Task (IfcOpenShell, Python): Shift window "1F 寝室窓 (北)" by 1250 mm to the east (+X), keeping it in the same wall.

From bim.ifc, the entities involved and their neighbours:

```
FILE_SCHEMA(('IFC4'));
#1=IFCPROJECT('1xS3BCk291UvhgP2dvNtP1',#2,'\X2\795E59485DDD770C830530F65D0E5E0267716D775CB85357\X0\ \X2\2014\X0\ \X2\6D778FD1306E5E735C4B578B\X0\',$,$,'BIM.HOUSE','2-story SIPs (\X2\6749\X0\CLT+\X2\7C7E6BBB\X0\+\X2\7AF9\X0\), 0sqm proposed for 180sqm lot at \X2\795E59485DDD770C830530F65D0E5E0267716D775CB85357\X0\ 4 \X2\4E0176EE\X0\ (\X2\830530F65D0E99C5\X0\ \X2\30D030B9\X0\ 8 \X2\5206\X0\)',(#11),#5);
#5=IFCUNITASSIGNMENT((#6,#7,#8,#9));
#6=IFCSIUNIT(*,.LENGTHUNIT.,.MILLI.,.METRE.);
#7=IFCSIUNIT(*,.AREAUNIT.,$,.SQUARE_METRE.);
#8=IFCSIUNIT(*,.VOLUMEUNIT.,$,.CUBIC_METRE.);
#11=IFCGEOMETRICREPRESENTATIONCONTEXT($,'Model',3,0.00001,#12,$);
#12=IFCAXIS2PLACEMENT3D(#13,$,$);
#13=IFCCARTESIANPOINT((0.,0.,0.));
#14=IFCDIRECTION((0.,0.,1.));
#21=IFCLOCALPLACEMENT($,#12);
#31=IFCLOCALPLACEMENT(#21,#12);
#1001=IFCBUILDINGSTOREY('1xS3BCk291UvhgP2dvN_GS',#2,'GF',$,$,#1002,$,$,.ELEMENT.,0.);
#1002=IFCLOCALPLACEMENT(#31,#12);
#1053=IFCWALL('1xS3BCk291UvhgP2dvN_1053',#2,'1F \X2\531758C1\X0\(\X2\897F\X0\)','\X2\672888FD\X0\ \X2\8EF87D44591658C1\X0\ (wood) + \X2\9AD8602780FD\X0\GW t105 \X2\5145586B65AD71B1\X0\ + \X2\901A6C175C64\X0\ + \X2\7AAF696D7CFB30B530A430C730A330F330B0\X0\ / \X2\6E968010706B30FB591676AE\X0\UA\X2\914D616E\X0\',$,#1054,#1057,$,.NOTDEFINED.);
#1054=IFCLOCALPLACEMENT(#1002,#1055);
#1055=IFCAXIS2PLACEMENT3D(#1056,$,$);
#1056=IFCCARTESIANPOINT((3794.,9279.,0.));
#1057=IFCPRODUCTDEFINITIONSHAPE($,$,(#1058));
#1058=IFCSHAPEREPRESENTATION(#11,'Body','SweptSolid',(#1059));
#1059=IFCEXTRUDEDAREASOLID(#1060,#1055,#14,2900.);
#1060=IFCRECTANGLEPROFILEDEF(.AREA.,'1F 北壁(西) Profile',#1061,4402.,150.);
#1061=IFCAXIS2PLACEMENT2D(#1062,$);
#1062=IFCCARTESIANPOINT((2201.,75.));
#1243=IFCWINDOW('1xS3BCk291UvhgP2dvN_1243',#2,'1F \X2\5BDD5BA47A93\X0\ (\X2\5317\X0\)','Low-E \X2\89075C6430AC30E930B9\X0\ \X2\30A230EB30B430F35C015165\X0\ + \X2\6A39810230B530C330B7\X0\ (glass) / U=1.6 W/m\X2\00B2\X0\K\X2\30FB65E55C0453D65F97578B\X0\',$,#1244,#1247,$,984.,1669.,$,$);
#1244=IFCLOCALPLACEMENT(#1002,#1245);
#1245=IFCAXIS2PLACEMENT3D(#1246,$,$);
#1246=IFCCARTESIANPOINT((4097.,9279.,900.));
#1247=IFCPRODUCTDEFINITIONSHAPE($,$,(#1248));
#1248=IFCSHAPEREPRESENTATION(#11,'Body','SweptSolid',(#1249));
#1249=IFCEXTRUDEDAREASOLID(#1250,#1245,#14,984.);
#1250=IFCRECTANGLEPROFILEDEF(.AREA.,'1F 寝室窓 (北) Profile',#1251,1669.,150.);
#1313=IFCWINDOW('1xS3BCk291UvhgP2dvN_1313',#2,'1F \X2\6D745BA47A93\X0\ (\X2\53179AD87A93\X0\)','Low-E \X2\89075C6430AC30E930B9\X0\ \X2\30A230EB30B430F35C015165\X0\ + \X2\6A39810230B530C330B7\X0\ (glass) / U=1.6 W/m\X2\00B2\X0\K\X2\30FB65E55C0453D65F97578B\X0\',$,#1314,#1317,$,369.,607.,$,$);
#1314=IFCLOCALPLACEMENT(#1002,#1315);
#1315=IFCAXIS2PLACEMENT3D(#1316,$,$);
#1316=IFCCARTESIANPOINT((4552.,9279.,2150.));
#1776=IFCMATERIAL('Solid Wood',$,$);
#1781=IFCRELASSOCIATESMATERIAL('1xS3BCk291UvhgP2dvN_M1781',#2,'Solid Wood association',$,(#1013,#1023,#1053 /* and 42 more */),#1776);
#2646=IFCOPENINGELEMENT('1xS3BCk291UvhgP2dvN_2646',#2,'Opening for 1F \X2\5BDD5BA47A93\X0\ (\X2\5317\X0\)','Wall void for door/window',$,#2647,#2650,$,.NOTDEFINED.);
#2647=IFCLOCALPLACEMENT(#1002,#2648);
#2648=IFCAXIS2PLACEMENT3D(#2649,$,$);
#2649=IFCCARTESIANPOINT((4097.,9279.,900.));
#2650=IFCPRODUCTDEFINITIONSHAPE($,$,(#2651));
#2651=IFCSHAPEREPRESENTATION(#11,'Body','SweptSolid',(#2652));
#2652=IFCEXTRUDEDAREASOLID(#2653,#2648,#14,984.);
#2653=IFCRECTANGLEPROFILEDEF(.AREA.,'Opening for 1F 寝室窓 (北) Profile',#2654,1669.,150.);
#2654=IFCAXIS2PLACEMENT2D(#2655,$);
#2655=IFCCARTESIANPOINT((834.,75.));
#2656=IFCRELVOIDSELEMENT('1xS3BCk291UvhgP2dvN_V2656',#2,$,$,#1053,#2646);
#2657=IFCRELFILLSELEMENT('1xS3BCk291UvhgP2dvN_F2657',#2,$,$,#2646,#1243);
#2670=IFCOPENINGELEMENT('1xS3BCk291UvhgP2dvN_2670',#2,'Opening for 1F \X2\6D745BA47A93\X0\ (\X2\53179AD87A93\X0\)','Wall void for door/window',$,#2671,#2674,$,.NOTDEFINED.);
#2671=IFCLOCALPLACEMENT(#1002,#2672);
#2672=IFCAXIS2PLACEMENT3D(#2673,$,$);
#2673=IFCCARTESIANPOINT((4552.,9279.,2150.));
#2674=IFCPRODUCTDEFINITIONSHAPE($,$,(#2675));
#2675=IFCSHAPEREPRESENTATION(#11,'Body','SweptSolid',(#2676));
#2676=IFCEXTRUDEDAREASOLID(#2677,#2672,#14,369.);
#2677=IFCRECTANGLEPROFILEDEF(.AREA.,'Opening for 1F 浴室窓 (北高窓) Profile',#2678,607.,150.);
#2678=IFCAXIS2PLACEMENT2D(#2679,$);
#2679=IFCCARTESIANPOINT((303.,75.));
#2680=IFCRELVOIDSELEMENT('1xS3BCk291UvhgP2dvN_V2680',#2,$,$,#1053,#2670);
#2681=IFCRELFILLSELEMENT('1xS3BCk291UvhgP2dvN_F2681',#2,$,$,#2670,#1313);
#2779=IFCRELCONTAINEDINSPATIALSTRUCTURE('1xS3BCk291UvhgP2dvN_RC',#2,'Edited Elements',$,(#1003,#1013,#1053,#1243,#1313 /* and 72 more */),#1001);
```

```python
import ifcopenshell
import ifcopenshell.api.geometry
import ifcopenshell.util.placement
import ifcopenshell.util.unit

model = ifcopenshell.open("bim.ifc")
unit_scale = ifcopenshell.util.unit.calculate_unit_scale(model)

window = model.by_guid("1xS3BCk291UvhgP2dvN_1243")
opening = window.FillsVoids[0].RelatingOpeningElement
wall = opening.VoidsElements[0].RelatingBuildingElement

wall_matrix = ifcopenshell.util.placement.get_local_placement(wall.ObjectPlacement)
shift = wall_matrix[:3, 0] * 1.25 / unit_scale
before = ifcopenshell.util.placement.get_local_placement(window.ObjectPlacement)[:3, 3].copy()

# The window is not placed relative to its opening, so move both.
for product in (opening, window):
    matrix = ifcopenshell.util.placement.get_local_placement(product.ObjectPlacement)
    matrix[:3, 3] += shift
    ifcopenshell.api.geometry.edit_object_placement(model, product=product, matrix=matrix, is_si=False)

after = ifcopenshell.util.placement.get_local_placement(window.ObjectPlacement)[:3, 3]
print("window moved by", (after - before).round(3) + 0.0)

model.write("bim_v2.ifc")
```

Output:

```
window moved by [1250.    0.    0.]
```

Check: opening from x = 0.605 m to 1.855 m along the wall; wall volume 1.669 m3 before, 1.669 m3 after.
